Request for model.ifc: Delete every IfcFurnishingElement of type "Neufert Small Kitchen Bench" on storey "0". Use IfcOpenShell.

First a look at what the model holds.

```python
import ifcopenshell
import ifcopenshell.util.element

model = ifcopenshell.open("model.ifc")
print(model.schema)
storey = next(s for s in model.by_type("IfcBuildingStorey") if s.Name == "0")
furniture = [e for e in ifcopenshell.util.element.get_decomposition(storey) if e.is_a("IfcFurnishingElement")]
seen = {}
for e in furniture:
    element_type = ifcopenshell.util.element.get_type(e)
    name = element_type.Name if element_type not in (None, e) else None
    seen[name] = seen.get(name, 0) + 1
for name, count in sorted(seen.items(), key=str):
    print(count, "x", name)
```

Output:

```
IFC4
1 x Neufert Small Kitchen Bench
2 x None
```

```python
import ifcopenshell
import ifcopenshell.api.root
import ifcopenshell.util.element

model = ifcopenshell.open("model.ifc")

storey = next(s for s in model.by_type("IfcBuildingStorey") if s.Name == "0")
furniture = [e for e in ifcopenshell.util.element.get_decomposition(storey) if e.is_a("IfcFurnishingElement")]
targets = [e for e in furniture if (t := ifcopenshell.util.element.get_type(e)) not in (None, e) and t.Name == "Neufert Small Kitchen Bench"]

for e in targets:
    ifcopenshell.api.root.remove_product(model, product=e)
print(len(targets), "removed")

model.write("model_edited.ifc")
```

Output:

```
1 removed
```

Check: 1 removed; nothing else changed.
